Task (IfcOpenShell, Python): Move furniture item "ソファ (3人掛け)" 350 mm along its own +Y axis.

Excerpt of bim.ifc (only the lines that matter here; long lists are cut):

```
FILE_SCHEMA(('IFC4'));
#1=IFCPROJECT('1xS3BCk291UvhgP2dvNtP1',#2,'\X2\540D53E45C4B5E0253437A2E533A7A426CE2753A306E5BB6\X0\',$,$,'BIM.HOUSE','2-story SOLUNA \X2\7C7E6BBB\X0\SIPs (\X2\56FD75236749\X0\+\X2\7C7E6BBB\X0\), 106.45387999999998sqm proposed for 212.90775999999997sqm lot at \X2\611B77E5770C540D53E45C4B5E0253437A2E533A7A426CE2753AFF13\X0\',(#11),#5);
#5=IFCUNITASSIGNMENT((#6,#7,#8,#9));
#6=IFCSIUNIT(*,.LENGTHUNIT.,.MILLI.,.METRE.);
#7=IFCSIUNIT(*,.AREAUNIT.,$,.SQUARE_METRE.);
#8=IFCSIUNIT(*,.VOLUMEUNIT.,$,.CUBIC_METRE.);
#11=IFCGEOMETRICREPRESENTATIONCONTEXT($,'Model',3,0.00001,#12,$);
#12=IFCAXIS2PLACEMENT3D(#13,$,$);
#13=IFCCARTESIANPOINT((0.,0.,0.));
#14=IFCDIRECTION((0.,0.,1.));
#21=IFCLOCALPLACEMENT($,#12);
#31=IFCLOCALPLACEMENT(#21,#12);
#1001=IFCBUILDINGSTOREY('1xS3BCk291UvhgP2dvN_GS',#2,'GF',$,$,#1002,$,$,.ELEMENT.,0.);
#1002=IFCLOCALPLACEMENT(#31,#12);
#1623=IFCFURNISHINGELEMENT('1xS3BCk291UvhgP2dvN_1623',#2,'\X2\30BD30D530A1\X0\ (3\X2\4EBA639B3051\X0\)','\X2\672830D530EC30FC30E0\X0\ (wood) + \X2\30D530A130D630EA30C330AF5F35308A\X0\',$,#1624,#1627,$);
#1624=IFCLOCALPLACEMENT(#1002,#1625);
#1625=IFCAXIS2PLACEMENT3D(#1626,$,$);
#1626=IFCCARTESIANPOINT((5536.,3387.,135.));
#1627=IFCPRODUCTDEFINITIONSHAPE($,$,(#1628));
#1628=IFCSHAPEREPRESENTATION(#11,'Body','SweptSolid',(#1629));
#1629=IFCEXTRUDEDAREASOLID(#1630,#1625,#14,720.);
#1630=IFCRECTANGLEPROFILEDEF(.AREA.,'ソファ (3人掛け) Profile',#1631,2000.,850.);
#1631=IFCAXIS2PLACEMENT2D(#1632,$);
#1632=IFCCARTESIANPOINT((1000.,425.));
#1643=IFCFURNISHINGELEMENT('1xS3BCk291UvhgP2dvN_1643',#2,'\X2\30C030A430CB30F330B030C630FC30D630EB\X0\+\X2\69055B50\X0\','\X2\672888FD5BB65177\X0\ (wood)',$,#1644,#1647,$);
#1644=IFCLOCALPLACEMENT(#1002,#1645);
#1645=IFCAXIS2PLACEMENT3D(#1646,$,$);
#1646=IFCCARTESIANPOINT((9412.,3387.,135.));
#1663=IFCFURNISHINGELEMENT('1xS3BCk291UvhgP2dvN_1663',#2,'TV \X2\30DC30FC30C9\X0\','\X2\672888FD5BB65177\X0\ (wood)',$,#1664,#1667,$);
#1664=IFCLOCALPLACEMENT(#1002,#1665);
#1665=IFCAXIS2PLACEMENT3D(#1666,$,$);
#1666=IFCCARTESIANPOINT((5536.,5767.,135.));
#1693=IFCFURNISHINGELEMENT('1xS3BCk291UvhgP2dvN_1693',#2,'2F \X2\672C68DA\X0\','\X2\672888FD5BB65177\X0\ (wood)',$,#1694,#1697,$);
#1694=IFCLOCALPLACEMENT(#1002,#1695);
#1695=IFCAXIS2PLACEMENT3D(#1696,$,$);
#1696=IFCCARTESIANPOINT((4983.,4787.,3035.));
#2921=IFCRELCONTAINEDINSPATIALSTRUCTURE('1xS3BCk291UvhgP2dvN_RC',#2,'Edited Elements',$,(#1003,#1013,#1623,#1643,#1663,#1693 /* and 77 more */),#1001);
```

```python
import ifcopenshell
import ifcopenshell.api.geometry
import ifcopenshell.util.placement

model = ifcopenshell.open("bim.ifc")

item = model.by_guid("1xS3BCk291UvhgP2dvN_1623")
matrix = ifcopenshell.util.placement.get_local_placement(item.ObjectPlacement)
matrix[:3, 3] += matrix[:3, 1] * 350.0
ifcopenshell.api.geometry.edit_object_placement(model, product=item, matrix=matrix, is_si=False)

print(ifcopenshell.util.placement.get_local_placement(item.ObjectPlacement).round(3) + 0.0)

model.write("bim_rev.ifc")
```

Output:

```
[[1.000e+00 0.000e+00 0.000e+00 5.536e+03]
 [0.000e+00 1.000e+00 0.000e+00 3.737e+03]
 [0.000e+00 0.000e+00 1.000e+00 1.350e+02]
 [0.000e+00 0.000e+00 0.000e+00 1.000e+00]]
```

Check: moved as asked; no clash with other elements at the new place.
